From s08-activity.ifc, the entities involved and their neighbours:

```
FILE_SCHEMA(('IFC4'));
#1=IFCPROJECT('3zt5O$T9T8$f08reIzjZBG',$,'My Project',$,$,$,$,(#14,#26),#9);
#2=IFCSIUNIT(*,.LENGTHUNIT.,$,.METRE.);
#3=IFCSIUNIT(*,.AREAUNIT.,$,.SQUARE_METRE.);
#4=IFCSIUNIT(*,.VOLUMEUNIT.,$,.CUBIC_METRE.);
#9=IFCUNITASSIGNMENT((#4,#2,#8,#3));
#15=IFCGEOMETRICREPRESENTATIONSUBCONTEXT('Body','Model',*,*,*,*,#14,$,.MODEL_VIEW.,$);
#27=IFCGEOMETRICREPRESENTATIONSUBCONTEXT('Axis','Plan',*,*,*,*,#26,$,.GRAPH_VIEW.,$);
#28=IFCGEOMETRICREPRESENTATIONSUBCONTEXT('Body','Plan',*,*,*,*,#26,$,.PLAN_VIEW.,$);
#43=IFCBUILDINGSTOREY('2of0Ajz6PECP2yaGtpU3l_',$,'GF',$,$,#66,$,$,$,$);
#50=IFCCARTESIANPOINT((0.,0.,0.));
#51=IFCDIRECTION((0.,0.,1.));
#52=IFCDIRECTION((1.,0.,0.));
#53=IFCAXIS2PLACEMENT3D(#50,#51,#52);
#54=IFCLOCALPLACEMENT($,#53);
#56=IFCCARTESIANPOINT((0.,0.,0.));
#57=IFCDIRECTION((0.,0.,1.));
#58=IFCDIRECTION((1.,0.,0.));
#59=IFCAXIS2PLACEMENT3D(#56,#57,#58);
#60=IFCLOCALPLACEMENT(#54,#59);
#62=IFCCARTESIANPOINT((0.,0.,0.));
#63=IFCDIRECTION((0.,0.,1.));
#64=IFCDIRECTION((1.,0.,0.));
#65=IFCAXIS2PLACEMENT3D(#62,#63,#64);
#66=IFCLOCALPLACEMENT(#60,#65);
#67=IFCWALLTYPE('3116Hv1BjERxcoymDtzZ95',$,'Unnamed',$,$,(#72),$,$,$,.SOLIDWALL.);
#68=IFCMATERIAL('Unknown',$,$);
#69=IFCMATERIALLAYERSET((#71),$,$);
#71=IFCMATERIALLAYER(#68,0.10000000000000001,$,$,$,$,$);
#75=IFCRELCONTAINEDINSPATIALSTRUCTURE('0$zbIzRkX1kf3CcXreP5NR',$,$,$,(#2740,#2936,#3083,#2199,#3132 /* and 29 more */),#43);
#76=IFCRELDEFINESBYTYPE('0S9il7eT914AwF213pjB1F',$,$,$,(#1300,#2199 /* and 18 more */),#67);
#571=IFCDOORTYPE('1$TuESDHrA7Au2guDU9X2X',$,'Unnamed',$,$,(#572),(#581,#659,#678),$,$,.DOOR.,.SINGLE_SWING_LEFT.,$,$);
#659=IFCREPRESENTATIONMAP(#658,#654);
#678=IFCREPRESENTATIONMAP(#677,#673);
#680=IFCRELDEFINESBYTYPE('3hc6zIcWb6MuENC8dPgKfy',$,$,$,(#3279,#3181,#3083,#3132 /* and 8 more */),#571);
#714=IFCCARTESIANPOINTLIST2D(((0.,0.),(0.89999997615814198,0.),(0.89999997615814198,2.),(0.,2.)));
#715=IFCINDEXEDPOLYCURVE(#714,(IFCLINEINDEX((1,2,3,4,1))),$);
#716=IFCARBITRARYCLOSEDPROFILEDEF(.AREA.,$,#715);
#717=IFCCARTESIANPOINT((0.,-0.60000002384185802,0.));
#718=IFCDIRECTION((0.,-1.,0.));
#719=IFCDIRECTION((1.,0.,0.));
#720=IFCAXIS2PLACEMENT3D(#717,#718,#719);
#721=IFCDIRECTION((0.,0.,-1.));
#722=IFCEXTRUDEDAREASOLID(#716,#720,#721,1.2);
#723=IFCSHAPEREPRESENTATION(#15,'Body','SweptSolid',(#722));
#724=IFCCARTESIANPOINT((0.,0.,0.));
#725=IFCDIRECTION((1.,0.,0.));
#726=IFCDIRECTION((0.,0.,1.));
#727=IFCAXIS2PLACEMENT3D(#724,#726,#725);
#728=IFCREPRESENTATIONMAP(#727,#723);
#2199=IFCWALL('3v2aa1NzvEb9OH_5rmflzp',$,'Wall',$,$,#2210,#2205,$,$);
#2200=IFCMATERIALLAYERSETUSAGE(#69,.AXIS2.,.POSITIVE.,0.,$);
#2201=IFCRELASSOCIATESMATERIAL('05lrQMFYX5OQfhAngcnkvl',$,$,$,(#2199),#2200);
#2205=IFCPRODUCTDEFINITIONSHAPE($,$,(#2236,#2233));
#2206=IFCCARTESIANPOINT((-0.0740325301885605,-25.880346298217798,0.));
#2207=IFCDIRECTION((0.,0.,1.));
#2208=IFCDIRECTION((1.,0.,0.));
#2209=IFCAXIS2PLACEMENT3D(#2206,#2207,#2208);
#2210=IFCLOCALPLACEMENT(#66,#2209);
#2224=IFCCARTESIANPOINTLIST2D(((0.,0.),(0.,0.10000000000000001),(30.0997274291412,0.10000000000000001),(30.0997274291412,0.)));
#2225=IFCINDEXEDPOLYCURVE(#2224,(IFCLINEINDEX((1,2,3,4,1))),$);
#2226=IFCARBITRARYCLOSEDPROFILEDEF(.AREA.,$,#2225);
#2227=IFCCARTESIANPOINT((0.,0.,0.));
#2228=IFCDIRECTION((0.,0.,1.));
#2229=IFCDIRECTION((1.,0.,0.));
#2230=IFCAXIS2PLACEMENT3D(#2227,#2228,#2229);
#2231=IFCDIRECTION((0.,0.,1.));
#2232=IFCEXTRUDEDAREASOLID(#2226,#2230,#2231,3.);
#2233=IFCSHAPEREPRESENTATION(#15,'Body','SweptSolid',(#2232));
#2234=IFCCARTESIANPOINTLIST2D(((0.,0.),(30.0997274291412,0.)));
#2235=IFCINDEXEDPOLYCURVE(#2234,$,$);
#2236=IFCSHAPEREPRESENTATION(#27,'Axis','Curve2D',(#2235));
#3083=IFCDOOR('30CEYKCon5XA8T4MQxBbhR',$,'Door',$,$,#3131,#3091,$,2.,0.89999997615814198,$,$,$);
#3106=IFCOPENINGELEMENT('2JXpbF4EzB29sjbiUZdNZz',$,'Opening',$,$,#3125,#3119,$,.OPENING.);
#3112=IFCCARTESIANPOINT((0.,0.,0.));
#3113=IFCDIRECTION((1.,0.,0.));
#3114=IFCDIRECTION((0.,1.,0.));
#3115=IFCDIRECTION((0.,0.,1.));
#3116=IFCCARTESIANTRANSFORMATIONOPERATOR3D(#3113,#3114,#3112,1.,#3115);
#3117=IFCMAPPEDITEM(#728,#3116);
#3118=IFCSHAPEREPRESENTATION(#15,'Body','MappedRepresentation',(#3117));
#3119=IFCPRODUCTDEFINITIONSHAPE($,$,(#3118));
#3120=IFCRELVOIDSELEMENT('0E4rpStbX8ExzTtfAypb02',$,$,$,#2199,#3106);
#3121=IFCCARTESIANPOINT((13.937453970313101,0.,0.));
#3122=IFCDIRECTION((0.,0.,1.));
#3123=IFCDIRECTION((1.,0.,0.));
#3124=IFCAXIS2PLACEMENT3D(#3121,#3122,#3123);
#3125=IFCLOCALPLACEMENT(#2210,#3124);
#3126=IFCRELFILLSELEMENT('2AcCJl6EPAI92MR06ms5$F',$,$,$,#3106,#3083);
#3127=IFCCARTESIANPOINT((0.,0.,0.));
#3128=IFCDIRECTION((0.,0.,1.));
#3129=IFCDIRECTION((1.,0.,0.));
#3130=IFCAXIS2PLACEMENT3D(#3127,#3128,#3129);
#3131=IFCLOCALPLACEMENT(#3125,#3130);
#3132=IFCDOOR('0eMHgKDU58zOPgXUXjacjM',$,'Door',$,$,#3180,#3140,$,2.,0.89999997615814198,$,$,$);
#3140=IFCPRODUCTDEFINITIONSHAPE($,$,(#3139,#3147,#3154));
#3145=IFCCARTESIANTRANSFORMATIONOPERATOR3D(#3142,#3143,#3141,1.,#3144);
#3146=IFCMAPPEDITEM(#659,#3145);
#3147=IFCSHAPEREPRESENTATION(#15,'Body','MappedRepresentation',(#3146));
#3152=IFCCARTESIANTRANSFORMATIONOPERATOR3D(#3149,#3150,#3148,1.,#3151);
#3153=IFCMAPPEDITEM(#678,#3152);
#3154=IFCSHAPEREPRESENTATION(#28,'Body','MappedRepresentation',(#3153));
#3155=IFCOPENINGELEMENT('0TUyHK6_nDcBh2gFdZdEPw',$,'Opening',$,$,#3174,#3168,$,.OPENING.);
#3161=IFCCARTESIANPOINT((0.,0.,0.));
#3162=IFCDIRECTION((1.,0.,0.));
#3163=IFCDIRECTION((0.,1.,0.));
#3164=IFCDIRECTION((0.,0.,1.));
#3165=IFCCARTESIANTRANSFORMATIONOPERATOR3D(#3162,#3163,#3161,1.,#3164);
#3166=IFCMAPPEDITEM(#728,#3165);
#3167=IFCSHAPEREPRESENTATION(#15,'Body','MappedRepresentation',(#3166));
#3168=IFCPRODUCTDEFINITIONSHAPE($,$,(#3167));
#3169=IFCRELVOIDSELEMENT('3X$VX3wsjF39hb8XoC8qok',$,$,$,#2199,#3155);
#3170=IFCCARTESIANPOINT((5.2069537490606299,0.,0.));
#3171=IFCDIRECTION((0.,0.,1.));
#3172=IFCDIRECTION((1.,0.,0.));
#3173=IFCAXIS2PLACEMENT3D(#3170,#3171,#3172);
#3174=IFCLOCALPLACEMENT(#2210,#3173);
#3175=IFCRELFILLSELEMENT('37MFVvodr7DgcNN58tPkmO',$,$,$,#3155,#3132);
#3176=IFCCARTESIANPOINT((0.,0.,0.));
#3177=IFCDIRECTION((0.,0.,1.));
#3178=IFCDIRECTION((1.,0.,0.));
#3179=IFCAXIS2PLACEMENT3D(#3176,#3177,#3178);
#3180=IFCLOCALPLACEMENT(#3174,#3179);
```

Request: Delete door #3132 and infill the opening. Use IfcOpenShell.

```python
import ifcopenshell
import ifcopenshell.api.feature
import ifcopenshell.api.root
import ifcopenshell.geom
import ifcopenshell.util.shape

model = ifcopenshell.open("s08-activity.ifc")
settings = ifcopenshell.geom.settings()


def volume(element):
    """Net volume in cubic metres, openings subtracted."""
    shape = ifcopenshell.geom.create_shape(settings, element)
    return ifcopenshell.util.shape.get_volume(shape.geometry)


door = model.by_guid("0eMHgKDU58zOPgXUXjacjM")
opening = door.FillsVoids[0].RelatingOpeningElement
wall = opening.VoidsElements[0].RelatingBuildingElement
before = volume(wall)

ifcopenshell.api.root.remove_product(model, product=door)
ifcopenshell.api.feature.remove_feature(model, feature=opening)

after = volume(wall)

print(f"wall volume {before:.3f} -> {after:.3f} m3")

model.write("s08-activity_updated.ifc")
```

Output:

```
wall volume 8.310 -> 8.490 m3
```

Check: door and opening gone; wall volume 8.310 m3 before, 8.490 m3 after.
